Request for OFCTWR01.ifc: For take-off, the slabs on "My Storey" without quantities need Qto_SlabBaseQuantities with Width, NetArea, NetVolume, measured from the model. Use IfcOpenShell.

First a look at what the model holds.

```python
import ifcopenshell
import ifcopenshell.util.element
import ifcopenshell.util.unit

model = ifcopenshell.open("OFCTWR01.ifc")
print(model.schema)
for unit_type in ("LENGTHUNIT", "AREAUNIT", "VOLUMEUNIT"):
    print(unit_type, ifcopenshell.util.unit.calculate_unit_scale(model, unit_type))
storey = next(s for s in model.by_type("IfcBuildingStorey") if s.Name == "My Storey")
slabs = [e for e in ifcopenshell.util.element.get_decomposition(storey) if e.is_a("IfcSlab")]
for e in sorted(slabs, key=lambda e: e.id()):
    print(e.id(), e.is_a(), e.Name, list(ifcopenshell.util.element.get_psets(e, qtos_only=True)), sep=" | ")
```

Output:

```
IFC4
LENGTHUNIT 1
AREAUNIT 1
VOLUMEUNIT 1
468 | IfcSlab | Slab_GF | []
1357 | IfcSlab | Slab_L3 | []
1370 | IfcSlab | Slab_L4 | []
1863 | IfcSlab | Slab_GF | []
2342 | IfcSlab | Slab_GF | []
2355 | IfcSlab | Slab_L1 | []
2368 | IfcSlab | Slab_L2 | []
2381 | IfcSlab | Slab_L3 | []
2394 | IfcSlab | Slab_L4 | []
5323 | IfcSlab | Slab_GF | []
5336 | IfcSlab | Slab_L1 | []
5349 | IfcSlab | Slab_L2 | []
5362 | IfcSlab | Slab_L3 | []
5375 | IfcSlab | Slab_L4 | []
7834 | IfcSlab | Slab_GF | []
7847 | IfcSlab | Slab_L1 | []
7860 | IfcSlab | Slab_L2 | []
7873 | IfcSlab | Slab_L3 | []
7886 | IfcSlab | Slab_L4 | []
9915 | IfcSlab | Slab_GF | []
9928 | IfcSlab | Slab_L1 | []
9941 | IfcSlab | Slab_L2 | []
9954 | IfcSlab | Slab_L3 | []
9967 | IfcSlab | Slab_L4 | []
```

```python
import ifcopenshell
import ifcopenshell.api.pset
import ifcopenshell.geom
import ifcopenshell.util.element
import ifcopenshell.util.shape
import ifcopenshell.util.unit

model = ifcopenshell.open("OFCTWR01.ifc")
unit_scale = ifcopenshell.util.unit.calculate_unit_scale(model)
area_scale = ifcopenshell.util.unit.calculate_unit_scale(model, "AREAUNIT")
volume_scale = ifcopenshell.util.unit.calculate_unit_scale(model, "VOLUMEUNIT")
settings = ifcopenshell.geom.settings()

storey = next(s for s in model.by_type("IfcBuildingStorey") if s.Name == "My Storey")
slabs = [e for e in ifcopenshell.util.element.get_decomposition(storey) if e.is_a("IfcSlab")]

for e in sorted(slabs, key=lambda e: e.id()):
    if ifcopenshell.util.element.get_psets(e, qtos_only=True, should_inherit=False):
        continue
    # Geometry comes back in metres, in the element's own axes.
    shape = ifcopenshell.geom.create_shape(settings, e)
    values = {
        "Width": ifcopenshell.util.shape.get_z(shape.geometry) / unit_scale,
        "NetArea": ifcopenshell.util.shape.get_footprint_area(shape.geometry) / area_scale,
        "NetVolume": ifcopenshell.util.shape.get_volume(shape.geometry) / volume_scale,
    }
    qto = ifcopenshell.api.pset.add_qto(model, product=e, name="Qto_SlabBaseQuantities")
    ifcopenshell.api.pset.edit_qto(model, qto=qto, properties=values)
    print(e.id(), {k: round(v, 3) for k, v in values.items()})

model.write("OFCTWR01-out.ifc")
```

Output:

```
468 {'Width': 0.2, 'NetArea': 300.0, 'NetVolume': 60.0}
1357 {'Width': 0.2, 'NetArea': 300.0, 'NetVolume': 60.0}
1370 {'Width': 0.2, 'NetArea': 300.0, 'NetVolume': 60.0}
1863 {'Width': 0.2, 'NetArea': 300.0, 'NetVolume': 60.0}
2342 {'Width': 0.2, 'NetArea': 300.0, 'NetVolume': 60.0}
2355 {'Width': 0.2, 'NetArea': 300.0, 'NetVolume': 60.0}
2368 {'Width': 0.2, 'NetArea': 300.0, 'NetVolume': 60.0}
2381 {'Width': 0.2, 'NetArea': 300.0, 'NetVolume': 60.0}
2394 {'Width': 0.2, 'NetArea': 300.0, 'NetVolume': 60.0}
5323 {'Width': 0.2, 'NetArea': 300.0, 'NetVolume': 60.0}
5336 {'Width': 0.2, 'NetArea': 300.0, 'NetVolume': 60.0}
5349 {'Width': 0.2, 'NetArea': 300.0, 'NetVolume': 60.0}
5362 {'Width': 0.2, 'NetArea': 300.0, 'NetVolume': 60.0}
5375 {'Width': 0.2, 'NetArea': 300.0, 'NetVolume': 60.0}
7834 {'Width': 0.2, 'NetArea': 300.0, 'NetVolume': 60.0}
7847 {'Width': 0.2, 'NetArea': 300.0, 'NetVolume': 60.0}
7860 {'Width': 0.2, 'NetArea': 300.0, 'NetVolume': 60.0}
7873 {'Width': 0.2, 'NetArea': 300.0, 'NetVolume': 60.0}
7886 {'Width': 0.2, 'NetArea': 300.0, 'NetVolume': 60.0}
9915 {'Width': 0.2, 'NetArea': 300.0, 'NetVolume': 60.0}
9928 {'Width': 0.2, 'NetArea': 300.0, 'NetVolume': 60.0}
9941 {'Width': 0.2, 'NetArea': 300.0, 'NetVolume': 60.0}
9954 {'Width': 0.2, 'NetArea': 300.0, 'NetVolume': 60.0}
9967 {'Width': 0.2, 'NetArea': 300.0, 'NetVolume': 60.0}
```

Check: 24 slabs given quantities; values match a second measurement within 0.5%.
